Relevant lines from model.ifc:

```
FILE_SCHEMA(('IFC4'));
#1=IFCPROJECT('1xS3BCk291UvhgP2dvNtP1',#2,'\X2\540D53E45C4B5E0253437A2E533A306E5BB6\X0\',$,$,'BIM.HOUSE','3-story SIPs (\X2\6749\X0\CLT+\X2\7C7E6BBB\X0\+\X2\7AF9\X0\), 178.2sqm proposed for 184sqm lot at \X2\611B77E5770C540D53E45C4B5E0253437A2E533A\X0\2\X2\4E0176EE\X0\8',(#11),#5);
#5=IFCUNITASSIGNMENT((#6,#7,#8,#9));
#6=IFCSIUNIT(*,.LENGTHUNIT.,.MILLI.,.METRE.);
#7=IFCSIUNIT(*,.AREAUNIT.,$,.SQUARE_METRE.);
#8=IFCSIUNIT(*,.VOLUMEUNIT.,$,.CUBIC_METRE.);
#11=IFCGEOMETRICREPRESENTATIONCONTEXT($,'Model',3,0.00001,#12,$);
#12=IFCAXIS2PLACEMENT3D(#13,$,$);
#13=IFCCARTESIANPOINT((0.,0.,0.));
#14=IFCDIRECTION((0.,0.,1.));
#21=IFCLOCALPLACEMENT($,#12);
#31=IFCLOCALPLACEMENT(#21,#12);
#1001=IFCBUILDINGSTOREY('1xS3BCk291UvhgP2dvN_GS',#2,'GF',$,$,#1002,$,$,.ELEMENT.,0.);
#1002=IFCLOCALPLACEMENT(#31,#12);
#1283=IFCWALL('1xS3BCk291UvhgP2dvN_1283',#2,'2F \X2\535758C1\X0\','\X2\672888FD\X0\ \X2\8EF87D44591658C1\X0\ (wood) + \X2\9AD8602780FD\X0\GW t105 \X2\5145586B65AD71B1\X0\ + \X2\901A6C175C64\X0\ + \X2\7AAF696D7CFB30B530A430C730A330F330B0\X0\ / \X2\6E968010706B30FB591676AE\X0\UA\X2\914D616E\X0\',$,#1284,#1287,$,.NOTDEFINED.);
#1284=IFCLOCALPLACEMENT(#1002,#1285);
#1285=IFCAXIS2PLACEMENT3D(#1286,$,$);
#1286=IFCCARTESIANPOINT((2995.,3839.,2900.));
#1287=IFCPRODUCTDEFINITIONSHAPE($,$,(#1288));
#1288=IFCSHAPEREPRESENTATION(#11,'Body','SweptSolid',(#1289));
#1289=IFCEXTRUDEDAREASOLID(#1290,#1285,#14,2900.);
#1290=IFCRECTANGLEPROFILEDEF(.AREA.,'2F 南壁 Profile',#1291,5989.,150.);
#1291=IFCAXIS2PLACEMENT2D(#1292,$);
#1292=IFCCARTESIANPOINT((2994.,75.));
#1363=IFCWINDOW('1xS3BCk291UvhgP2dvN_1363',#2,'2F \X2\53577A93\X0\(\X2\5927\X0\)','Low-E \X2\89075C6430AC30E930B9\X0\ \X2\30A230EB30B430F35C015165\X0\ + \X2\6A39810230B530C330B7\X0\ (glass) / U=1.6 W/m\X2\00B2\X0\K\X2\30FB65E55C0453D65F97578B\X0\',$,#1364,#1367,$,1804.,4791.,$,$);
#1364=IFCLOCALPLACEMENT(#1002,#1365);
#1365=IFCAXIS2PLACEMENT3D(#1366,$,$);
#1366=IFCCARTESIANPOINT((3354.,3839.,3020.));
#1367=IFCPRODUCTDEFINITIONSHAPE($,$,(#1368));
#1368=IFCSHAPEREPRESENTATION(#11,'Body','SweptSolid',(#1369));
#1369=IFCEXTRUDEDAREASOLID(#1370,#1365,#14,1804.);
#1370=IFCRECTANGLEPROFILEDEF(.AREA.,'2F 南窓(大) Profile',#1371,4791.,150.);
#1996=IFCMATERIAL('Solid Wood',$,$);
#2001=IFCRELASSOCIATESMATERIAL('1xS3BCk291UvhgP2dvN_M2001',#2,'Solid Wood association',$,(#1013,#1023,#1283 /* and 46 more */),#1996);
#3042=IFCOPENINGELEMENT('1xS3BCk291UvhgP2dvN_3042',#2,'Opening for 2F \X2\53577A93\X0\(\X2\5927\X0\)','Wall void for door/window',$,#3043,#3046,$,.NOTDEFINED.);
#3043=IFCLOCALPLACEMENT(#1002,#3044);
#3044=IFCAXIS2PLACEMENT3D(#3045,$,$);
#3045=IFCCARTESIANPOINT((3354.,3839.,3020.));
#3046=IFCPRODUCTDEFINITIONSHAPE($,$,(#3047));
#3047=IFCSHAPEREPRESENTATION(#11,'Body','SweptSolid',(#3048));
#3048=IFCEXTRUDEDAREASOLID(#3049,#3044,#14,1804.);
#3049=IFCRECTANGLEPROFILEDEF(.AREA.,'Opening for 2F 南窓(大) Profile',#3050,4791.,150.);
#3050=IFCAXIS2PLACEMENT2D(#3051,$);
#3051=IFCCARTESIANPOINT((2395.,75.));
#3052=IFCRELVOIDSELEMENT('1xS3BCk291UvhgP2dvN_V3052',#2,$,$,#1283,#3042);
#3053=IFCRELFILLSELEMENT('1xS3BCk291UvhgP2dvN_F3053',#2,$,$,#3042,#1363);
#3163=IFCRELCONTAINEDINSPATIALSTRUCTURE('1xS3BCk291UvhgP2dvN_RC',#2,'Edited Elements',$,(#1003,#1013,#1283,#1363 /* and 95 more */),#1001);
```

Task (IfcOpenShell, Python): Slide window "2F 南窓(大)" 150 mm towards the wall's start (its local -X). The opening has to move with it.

```python
import ifcopenshell
import ifcopenshell.api.geometry
import ifcopenshell.util.placement

model = ifcopenshell.open("model.ifc")

window = model.by_id(1363)
opening = window.FillsVoids[0].RelatingOpeningElement
wall = opening.VoidsElements[0].RelatingBuildingElement

wall_matrix = ifcopenshell.util.placement.get_local_placement(wall.ObjectPlacement)
shift = wall_matrix[:3, 0] * -150.0
before = ifcopenshell.util.placement.get_local_placement(window.ObjectPlacement)[:3, 3].copy()

# The window is not placed relative to its opening, so move both.
for product in (opening, window):
    matrix = ifcopenshell.util.placement.get_local_placement(product.ObjectPlacement)
    matrix[:3, 3] += shift
    ifcopenshell.api.geometry.edit_object_placement(model, product=product, matrix=matrix, is_si=False)

after = ifcopenshell.util.placement.get_local_placement(window.ObjectPlacement)[:3, 3]
print("window moved by", (after - before).round(3) + 0.0)

model.write("model-out.ifc")
```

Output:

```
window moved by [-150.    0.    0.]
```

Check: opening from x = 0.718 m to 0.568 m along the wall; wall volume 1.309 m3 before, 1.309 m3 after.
